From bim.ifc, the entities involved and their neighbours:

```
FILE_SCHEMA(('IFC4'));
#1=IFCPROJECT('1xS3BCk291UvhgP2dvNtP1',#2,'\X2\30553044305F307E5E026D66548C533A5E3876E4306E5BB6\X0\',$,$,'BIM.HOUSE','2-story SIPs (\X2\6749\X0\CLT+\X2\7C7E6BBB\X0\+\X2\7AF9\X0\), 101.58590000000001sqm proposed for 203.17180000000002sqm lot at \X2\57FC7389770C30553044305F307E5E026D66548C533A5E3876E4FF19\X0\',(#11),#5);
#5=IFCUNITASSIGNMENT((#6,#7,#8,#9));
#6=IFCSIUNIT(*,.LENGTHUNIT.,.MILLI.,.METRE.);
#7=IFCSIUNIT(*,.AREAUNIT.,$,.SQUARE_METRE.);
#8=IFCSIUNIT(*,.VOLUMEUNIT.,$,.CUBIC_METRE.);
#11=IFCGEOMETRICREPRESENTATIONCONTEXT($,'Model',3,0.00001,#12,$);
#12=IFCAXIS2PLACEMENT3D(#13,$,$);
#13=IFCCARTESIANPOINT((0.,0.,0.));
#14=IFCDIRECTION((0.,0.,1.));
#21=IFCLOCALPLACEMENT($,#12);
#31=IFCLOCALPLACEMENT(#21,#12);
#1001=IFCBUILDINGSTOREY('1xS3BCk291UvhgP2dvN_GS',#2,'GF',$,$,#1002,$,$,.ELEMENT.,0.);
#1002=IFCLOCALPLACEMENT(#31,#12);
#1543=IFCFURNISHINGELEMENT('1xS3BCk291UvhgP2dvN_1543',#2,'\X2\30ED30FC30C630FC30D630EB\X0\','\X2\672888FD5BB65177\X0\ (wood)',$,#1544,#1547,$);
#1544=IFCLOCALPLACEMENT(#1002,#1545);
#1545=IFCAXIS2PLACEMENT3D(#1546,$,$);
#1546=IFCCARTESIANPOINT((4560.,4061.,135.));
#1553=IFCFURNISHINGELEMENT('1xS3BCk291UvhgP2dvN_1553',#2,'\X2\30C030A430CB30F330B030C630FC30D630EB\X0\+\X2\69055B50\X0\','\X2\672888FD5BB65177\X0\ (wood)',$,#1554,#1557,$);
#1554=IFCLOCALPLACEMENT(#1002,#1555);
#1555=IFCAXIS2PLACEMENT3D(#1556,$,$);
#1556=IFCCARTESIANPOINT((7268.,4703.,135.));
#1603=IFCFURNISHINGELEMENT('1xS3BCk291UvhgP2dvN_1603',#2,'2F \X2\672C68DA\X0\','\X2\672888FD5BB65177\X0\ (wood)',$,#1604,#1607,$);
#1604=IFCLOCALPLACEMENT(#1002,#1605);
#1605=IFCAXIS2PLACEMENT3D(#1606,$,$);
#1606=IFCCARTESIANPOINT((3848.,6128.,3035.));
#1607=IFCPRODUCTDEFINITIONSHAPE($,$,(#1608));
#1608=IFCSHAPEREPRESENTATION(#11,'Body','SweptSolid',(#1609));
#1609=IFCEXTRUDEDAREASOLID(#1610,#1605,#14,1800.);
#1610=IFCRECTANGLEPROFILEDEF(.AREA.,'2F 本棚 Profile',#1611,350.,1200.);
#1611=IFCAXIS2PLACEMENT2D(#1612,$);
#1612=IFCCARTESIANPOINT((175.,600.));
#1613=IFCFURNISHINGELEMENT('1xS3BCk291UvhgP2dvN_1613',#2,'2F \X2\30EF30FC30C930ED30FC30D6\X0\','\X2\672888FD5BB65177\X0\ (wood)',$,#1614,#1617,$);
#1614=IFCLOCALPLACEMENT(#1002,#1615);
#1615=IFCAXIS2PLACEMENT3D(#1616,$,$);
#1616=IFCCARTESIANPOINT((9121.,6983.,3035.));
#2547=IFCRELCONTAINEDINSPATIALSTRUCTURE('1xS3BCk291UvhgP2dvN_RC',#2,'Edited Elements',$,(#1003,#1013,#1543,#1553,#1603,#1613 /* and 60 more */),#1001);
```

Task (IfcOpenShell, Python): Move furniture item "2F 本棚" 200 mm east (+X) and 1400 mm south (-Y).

```python
import ifcopenshell
import ifcopenshell.api.geometry
import ifcopenshell.util.placement
import ifcopenshell.util.unit

model = ifcopenshell.open("bim.ifc")
unit_scale = ifcopenshell.util.unit.calculate_unit_scale(model)

item = model.by_guid("1xS3BCk291UvhgP2dvN_1603")
matrix = ifcopenshell.util.placement.get_local_placement(item.ObjectPlacement)
matrix[0, 3] += 0.2 / unit_scale
matrix[1, 3] -= 1.4 / unit_scale
ifcopenshell.api.geometry.edit_object_placement(model, product=item, matrix=matrix, is_si=False)

print(ifcopenshell.util.placement.get_local_placement(item.ObjectPlacement).round(3) + 0.0)

model.write("bim-out.ifc")
```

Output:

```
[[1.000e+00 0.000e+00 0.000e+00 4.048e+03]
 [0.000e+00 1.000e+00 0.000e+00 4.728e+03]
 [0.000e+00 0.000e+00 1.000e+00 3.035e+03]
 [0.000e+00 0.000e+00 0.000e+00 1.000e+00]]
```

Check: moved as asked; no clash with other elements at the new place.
